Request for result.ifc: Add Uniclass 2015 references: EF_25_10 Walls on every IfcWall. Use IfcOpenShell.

First a look at what the model holds.

```python
import ifcopenshell

model = ifcopenshell.open("result.ifc")
print(model.schema)
print("classifications:", [c.Name for c in model.by_type("IfcClassification")])
for ifc_class in ("IfcDoor", "IfcRoof", "IfcStair", "IfcWall", "IfcWindow"):
    print(ifc_class, len(model.by_type(ifc_class)))
```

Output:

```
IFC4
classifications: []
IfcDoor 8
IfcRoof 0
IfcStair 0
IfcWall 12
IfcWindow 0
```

```python
import ifcopenshell
import ifcopenshell.api.classification

model = ifcopenshell.open("result.ifc")

system = ifcopenshell.api.classification.add_classification(model, classification="Uniclass 2015")

codes = {
    "IfcWall": ("EF_25_10", "Walls"),
}
for ifc_class, (code, name) in codes.items():
    products = model.by_type(ifc_class)
    ifcopenshell.api.classification.add_reference(
        model, products=products, classification=system, identification=code, name=name
    )
    print(code, len(products))

model.write("result_edited.ifc")
```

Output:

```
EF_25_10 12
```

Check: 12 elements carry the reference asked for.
